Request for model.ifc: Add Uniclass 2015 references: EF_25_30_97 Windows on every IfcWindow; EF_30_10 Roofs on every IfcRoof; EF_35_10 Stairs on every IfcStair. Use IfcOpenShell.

First a look at what the model holds.

```python
import ifcopenshell

model = ifcopenshell.open("model.ifc")
print(model.schema)
print("classifications:", [c.Name for c in model.by_type("IfcClassification")])
for ifc_class in ("IfcDoor", "IfcRoof", "IfcStair", "IfcWall", "IfcWindow"):
    print(ifc_class, len(model.by_type(ifc_class)))
```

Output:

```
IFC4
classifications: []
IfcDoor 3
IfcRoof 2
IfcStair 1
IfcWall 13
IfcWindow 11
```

```python
import ifcopenshell
import ifcopenshell.api.classification

model = ifcopenshell.open("model.ifc")

system = ifcopenshell.api.classification.add_classification(model, classification="Uniclass 2015")

codes = {
    "IfcWindow": ("EF_25_30_97", "Windows"),
    "IfcRoof": ("EF_30_10", "Roofs"),
    "IfcStair": ("EF_35_10", "Stairs"),
}
for ifc_class, (code, name) in codes.items():
    products = model.by_type(ifc_class)
    ifcopenshell.api.classification.add_reference(
        model, products=products, classification=system, identification=code, name=name
    )
    print(code, len(products))

model.write("model_updated.ifc")
```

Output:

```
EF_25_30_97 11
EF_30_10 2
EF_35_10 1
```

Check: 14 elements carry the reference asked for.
